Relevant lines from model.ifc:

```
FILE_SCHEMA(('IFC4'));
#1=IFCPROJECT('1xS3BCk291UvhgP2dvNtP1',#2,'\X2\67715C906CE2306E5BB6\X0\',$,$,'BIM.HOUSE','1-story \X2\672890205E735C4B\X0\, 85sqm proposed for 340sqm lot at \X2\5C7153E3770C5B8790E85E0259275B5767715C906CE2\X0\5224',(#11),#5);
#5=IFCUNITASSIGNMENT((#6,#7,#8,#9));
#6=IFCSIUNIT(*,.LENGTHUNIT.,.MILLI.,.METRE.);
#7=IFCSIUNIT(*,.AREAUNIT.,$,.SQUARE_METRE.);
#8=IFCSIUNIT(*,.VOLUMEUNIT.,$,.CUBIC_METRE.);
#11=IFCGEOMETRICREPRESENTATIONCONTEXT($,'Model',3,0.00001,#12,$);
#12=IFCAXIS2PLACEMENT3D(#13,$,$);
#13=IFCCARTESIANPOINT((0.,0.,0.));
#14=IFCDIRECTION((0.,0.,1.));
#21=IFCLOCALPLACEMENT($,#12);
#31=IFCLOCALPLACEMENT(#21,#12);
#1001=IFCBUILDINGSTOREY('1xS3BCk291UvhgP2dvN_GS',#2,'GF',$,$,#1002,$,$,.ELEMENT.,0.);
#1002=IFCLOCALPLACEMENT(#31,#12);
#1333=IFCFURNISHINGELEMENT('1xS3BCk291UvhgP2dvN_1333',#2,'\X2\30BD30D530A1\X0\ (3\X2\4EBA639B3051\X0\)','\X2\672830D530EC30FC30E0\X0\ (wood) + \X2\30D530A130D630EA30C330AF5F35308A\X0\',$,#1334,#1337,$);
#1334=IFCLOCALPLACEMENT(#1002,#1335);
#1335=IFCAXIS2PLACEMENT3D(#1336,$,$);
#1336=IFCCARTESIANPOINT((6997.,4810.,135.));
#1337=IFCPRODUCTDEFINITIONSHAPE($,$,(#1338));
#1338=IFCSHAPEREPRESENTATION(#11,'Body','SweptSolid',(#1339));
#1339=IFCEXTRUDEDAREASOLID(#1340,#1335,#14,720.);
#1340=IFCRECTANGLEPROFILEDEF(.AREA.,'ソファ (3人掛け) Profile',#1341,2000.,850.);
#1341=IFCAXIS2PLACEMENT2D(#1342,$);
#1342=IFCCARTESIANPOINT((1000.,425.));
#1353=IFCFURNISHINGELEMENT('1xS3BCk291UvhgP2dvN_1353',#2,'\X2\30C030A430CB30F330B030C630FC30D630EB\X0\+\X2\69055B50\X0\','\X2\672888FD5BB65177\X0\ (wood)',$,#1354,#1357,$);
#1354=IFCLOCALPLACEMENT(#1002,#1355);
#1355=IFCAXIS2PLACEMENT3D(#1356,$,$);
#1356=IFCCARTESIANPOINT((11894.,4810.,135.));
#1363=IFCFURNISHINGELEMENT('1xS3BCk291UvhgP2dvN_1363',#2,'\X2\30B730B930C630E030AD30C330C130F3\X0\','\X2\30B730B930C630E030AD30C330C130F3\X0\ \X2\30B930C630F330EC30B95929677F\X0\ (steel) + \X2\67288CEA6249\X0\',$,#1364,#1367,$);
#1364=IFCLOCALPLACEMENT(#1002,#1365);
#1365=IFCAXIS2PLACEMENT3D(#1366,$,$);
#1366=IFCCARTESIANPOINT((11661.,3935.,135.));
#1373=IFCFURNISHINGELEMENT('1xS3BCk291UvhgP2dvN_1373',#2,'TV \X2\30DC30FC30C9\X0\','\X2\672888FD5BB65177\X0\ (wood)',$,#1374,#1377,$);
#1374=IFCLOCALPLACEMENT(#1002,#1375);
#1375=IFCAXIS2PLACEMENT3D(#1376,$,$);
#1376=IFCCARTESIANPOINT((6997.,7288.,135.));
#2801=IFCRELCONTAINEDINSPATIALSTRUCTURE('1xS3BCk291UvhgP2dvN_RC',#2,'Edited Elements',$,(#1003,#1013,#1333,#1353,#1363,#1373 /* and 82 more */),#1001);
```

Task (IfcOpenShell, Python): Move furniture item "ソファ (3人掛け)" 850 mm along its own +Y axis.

```python
import ifcopenshell
import ifcopenshell.api.geometry
import ifcopenshell.util.placement

model = ifcopenshell.open("model.ifc")

item = model.by_guid("1xS3BCk291UvhgP2dvN_1333")
matrix = ifcopenshell.util.placement.get_local_placement(item.ObjectPlacement)
matrix[:3, 3] += matrix[:3, 1] * 850.0
ifcopenshell.api.geometry.edit_object_placement(model, product=item, matrix=matrix, is_si=False)

print(ifcopenshell.util.placement.get_local_placement(item.ObjectPlacement).round(3) + 0.0)

model.write("model-out.ifc")
```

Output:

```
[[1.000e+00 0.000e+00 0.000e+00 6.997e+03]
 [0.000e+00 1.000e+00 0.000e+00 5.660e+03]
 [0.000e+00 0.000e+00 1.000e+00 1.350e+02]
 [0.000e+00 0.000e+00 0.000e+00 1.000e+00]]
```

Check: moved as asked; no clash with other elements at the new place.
